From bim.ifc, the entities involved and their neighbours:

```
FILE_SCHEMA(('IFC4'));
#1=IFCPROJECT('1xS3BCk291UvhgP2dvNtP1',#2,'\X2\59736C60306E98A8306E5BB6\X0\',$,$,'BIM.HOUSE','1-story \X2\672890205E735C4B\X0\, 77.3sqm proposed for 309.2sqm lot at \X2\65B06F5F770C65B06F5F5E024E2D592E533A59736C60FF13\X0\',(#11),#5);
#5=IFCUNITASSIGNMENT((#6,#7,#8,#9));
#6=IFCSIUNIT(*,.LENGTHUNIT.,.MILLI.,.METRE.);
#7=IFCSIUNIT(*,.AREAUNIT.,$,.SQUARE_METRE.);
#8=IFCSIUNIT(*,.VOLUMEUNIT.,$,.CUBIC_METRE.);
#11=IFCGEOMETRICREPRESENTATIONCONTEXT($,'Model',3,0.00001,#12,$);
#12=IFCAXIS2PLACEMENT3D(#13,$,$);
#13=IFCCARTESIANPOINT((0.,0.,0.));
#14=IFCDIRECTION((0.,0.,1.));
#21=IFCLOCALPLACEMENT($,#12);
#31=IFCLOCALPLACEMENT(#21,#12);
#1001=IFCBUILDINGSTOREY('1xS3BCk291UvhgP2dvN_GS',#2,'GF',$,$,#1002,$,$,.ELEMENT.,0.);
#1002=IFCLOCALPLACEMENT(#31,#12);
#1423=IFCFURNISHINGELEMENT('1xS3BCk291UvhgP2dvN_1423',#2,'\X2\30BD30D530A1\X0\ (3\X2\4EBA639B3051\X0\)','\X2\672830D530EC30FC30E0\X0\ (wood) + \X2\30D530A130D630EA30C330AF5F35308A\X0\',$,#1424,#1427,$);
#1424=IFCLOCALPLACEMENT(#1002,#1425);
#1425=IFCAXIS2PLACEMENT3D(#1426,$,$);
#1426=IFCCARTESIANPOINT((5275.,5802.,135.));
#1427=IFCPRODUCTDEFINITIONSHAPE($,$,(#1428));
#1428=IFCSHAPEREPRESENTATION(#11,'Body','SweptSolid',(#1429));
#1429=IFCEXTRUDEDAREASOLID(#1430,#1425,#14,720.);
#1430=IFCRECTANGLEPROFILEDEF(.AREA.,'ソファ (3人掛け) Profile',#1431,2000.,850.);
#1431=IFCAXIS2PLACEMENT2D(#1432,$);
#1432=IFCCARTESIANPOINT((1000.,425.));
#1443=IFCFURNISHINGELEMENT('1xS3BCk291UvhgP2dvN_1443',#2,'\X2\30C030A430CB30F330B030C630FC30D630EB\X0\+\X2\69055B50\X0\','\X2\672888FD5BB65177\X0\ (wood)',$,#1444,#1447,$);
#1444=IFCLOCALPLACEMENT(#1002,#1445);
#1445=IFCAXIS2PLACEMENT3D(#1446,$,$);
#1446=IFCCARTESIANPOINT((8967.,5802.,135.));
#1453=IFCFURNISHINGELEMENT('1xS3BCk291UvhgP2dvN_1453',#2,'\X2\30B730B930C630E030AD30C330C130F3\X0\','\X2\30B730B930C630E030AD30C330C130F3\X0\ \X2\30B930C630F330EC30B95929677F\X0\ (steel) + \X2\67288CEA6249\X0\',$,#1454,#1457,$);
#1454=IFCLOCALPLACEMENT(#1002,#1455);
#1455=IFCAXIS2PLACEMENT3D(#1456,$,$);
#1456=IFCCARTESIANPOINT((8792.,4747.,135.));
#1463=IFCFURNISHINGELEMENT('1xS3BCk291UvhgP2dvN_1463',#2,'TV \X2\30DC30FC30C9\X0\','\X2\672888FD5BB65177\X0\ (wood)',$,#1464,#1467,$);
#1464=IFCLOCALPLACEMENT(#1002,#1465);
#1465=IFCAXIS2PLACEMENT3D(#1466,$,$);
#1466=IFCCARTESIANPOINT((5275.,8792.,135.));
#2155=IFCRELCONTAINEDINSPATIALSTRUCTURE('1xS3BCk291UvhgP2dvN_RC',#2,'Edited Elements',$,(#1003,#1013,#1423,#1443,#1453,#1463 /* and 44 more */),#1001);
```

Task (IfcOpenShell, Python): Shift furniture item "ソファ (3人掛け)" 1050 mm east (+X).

```python
import ifcopenshell
import ifcopenshell.api.geometry
import ifcopenshell.util.placement
import ifcopenshell.util.unit

model = ifcopenshell.open("bim.ifc")
unit_scale = ifcopenshell.util.unit.calculate_unit_scale(model)

item = model.by_guid("1xS3BCk291UvhgP2dvN_1423")
matrix = ifcopenshell.util.placement.get_local_placement(item.ObjectPlacement)
matrix[0, 3] += 1.05 / unit_scale
ifcopenshell.api.geometry.edit_object_placement(model, product=item, matrix=matrix, is_si=False)

print(ifcopenshell.util.placement.get_local_placement(item.ObjectPlacement).round(3) + 0.0)

model.write("bim-out.ifc")
```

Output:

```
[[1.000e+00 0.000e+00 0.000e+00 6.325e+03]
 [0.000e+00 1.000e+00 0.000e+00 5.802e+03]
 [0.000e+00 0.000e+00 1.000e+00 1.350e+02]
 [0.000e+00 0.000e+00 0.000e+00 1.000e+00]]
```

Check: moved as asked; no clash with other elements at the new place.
